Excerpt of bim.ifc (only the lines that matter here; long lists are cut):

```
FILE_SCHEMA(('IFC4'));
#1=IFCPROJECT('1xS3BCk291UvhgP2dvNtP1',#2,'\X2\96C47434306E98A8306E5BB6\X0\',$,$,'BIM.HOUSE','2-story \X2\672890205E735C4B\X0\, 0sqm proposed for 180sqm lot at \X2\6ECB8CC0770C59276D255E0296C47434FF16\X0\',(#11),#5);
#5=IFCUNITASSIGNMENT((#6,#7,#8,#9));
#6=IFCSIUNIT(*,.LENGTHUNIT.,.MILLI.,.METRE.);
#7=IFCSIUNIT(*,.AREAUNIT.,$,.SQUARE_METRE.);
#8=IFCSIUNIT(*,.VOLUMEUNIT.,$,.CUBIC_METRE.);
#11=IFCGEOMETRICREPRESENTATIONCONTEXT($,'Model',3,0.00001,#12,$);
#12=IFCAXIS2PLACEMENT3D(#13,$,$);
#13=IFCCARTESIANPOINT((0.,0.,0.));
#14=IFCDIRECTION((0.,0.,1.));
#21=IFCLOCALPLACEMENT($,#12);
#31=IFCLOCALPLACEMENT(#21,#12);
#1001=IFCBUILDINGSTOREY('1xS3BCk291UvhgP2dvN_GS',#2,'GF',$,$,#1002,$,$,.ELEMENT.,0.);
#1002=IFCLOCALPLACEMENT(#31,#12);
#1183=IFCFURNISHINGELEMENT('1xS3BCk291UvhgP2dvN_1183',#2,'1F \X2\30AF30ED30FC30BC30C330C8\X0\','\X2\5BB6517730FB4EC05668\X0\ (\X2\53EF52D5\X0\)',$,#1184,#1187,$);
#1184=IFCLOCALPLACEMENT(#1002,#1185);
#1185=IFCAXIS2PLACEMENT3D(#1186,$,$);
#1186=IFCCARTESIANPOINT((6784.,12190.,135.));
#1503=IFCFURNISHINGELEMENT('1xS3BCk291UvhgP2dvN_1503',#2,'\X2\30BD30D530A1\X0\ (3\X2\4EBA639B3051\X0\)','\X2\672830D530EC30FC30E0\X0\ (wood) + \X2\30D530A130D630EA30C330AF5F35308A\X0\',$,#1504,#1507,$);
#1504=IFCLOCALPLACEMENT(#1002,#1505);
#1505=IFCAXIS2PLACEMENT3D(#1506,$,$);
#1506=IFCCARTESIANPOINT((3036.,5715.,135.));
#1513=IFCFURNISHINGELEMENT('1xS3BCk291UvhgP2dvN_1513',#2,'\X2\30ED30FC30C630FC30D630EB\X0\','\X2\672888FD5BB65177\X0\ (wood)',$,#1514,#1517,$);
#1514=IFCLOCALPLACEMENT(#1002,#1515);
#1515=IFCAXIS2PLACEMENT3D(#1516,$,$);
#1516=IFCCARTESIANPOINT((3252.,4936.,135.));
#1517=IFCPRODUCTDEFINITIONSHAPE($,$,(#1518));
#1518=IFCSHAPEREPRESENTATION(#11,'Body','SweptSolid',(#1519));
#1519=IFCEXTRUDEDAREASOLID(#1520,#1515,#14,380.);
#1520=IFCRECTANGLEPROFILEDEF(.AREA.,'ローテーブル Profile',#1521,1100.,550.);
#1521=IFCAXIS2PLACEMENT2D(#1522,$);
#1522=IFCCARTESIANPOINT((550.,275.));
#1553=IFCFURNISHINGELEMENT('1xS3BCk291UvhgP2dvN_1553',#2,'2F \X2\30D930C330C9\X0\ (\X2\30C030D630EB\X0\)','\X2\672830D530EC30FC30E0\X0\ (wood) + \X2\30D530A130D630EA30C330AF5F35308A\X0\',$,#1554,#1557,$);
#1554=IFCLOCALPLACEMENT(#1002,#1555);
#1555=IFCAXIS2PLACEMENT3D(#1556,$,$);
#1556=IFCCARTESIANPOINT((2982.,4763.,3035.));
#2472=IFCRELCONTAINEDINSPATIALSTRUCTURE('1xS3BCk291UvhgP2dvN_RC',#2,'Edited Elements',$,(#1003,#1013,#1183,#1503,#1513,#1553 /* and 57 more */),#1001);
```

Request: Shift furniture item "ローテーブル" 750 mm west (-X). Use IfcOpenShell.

```python
import ifcopenshell
import ifcopenshell.api.geometry
import ifcopenshell.util.placement
import ifcopenshell.util.unit

model = ifcopenshell.open("bim.ifc")
unit_scale = ifcopenshell.util.unit.calculate_unit_scale(model)

item = model.by_guid("1xS3BCk291UvhgP2dvN_1513")
matrix = ifcopenshell.util.placement.get_local_placement(item.ObjectPlacement)
matrix[0, 3] -= 0.75 / unit_scale
ifcopenshell.api.geometry.edit_object_placement(model, product=item, matrix=matrix, is_si=False)

print(ifcopenshell.util.placement.get_local_placement(item.ObjectPlacement).round(3) + 0.0)

model.write("bim_rev.ifc")
```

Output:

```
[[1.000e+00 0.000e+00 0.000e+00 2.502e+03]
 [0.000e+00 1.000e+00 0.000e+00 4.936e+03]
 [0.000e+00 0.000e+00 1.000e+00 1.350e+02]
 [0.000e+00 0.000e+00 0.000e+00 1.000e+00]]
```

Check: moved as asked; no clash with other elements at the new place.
